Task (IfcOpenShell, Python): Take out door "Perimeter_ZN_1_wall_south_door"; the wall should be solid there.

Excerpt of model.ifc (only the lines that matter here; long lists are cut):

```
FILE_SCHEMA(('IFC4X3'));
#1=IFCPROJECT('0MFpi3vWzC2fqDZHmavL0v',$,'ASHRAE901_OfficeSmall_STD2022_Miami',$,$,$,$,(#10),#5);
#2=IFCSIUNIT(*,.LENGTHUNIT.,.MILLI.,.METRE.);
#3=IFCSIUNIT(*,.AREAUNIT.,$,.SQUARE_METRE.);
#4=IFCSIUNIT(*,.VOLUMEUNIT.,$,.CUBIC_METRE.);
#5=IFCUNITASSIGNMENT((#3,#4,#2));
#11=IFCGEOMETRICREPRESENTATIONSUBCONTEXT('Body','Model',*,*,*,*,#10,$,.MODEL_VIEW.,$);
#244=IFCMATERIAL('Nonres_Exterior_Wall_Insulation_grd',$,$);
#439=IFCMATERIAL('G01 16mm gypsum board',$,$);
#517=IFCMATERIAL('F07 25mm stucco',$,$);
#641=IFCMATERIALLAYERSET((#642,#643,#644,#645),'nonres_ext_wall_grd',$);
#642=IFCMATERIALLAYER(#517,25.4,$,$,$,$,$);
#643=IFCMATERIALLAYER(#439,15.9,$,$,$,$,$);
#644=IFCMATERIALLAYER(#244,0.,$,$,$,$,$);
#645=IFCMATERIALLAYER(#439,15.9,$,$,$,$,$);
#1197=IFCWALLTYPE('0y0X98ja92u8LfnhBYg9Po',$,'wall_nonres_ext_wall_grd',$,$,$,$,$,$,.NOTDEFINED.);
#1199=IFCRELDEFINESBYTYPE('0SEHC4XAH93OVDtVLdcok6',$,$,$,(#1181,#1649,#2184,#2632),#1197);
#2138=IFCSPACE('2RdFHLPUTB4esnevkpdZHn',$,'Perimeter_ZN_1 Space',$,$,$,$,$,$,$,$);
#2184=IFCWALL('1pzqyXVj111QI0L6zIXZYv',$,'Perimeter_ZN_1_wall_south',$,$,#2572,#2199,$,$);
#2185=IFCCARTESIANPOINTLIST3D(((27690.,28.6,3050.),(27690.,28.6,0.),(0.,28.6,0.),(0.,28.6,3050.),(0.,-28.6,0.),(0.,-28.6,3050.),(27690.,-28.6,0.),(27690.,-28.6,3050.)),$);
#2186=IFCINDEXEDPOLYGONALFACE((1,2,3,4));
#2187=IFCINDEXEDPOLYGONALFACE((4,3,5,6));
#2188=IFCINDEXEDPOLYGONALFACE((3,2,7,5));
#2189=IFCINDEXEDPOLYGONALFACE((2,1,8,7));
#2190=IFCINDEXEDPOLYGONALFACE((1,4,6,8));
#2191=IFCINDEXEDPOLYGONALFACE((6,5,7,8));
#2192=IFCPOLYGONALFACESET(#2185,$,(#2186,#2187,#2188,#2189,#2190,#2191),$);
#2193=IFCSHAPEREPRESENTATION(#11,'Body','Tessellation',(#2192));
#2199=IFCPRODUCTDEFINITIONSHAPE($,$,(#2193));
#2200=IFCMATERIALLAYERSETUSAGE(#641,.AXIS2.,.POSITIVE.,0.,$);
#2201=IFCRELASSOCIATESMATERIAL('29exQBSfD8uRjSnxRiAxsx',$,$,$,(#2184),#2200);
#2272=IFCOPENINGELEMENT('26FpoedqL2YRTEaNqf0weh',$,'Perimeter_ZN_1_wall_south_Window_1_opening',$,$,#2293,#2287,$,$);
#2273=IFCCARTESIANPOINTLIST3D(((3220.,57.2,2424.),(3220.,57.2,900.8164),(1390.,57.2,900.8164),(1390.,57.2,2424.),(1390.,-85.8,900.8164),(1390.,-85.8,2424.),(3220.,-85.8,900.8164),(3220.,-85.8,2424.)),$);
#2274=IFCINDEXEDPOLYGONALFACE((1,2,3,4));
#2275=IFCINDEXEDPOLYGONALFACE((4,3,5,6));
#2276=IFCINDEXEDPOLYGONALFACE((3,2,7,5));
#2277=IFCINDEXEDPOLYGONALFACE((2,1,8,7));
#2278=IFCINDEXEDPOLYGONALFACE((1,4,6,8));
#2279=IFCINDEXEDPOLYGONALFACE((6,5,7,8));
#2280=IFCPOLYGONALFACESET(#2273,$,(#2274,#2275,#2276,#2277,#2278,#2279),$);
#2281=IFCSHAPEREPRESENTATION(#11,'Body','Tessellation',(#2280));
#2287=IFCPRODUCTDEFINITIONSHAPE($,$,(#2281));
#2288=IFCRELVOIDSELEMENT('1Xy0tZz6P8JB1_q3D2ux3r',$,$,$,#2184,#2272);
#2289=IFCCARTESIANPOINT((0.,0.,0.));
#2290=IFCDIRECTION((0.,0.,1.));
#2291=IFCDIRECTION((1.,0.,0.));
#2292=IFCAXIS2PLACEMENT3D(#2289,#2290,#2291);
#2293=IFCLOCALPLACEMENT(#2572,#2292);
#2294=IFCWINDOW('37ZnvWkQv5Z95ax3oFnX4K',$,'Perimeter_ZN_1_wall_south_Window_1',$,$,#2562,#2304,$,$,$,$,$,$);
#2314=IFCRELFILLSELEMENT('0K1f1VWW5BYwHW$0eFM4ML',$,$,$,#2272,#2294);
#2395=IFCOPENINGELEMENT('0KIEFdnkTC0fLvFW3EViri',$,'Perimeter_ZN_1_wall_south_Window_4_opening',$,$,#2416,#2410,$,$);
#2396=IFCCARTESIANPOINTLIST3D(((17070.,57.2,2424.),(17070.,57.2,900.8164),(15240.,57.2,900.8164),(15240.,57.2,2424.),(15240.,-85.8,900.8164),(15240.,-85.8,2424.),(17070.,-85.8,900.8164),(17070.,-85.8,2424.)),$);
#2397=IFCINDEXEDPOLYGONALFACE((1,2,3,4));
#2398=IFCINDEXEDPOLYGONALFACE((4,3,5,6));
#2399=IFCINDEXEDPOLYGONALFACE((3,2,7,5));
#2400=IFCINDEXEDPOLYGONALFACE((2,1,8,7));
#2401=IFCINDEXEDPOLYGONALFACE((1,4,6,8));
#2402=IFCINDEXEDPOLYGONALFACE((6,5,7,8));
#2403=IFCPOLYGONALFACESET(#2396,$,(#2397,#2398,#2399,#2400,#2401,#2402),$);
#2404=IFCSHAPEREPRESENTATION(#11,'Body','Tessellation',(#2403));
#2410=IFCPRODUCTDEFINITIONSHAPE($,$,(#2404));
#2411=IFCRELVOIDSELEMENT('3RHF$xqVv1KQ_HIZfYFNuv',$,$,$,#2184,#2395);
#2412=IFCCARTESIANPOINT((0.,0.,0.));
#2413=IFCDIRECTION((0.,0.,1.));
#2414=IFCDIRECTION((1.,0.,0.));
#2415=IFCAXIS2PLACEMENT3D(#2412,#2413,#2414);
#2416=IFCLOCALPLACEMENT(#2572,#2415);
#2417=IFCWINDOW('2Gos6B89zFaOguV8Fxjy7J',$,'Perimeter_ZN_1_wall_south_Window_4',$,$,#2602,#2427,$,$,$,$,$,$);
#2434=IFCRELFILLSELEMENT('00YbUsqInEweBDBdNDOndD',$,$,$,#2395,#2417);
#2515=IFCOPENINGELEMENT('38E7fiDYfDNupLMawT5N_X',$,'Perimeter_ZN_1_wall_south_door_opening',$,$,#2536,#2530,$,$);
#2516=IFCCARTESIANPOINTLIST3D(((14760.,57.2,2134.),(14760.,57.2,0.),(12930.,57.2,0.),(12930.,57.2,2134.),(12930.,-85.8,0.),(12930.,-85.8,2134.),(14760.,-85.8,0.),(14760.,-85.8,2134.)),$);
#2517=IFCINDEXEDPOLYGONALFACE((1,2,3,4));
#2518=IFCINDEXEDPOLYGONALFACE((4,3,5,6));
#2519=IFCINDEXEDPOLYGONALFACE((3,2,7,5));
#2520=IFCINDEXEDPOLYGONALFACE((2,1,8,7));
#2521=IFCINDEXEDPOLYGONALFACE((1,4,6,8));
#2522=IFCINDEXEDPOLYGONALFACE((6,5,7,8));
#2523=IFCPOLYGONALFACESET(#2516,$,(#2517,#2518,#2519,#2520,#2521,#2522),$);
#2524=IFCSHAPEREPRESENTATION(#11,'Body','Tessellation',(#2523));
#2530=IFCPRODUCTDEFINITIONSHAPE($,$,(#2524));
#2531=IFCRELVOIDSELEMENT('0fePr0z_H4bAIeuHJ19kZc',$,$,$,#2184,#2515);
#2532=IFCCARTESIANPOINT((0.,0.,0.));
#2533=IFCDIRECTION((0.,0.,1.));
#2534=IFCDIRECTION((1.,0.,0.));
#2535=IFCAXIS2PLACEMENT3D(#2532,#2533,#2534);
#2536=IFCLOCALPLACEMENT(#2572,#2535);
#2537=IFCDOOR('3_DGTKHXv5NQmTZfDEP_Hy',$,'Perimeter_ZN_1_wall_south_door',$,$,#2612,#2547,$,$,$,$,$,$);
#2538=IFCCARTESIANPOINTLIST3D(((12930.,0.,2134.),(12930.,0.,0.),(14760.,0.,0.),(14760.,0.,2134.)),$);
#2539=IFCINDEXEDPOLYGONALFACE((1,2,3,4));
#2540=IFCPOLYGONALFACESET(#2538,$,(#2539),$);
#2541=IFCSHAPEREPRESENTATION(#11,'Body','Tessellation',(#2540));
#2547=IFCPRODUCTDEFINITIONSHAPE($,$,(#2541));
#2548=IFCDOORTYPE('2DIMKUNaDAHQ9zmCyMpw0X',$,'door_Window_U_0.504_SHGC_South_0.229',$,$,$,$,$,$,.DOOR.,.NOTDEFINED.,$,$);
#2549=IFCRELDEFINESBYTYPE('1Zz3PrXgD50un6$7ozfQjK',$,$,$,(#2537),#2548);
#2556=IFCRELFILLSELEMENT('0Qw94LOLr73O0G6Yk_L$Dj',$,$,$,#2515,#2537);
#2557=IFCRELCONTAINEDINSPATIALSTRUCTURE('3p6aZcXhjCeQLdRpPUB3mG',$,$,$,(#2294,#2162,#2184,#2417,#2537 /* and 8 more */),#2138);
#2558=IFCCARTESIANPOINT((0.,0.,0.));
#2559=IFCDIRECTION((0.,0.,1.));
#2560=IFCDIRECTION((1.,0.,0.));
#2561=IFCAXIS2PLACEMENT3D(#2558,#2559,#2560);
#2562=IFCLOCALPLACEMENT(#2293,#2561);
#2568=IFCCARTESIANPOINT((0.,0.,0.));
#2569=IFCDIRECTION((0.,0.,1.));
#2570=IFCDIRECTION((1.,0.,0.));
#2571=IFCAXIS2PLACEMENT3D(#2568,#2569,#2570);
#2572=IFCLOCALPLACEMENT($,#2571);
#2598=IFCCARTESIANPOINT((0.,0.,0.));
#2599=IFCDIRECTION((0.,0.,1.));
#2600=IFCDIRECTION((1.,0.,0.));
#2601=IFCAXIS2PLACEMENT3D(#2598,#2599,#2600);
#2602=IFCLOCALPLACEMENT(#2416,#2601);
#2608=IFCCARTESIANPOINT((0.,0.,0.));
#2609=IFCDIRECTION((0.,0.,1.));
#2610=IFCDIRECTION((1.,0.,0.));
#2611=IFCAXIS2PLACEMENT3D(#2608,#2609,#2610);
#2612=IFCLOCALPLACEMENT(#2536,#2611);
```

```python
import ifcopenshell
import ifcopenshell.api.feature
import ifcopenshell.api.root
import ifcopenshell.geom
import ifcopenshell.util.shape

model = ifcopenshell.open("model.ifc")
settings = ifcopenshell.geom.settings()


def volume(element):
    """Net volume in cubic metres, openings subtracted."""
    shape = ifcopenshell.geom.create_shape(settings, element)
    return ifcopenshell.util.shape.get_volume(shape.geometry)


door = model.by_guid("3_DGTKHXv5NQmTZfDEP_Hy")
opening = door.FillsVoids[0].RelatingOpeningElement
wall = opening.VoidsElements[0].RelatingBuildingElement
before = volume(wall)

ifcopenshell.api.root.remove_product(model, product=door)
ifcopenshell.api.feature.remove_feature(model, feature=opening)

after = volume(wall)

print(f"wall volume {before:.3f} -> {after:.3f} m3")

model.write("model_updated.ifc")
```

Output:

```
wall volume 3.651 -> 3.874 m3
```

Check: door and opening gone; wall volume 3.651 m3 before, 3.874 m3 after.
